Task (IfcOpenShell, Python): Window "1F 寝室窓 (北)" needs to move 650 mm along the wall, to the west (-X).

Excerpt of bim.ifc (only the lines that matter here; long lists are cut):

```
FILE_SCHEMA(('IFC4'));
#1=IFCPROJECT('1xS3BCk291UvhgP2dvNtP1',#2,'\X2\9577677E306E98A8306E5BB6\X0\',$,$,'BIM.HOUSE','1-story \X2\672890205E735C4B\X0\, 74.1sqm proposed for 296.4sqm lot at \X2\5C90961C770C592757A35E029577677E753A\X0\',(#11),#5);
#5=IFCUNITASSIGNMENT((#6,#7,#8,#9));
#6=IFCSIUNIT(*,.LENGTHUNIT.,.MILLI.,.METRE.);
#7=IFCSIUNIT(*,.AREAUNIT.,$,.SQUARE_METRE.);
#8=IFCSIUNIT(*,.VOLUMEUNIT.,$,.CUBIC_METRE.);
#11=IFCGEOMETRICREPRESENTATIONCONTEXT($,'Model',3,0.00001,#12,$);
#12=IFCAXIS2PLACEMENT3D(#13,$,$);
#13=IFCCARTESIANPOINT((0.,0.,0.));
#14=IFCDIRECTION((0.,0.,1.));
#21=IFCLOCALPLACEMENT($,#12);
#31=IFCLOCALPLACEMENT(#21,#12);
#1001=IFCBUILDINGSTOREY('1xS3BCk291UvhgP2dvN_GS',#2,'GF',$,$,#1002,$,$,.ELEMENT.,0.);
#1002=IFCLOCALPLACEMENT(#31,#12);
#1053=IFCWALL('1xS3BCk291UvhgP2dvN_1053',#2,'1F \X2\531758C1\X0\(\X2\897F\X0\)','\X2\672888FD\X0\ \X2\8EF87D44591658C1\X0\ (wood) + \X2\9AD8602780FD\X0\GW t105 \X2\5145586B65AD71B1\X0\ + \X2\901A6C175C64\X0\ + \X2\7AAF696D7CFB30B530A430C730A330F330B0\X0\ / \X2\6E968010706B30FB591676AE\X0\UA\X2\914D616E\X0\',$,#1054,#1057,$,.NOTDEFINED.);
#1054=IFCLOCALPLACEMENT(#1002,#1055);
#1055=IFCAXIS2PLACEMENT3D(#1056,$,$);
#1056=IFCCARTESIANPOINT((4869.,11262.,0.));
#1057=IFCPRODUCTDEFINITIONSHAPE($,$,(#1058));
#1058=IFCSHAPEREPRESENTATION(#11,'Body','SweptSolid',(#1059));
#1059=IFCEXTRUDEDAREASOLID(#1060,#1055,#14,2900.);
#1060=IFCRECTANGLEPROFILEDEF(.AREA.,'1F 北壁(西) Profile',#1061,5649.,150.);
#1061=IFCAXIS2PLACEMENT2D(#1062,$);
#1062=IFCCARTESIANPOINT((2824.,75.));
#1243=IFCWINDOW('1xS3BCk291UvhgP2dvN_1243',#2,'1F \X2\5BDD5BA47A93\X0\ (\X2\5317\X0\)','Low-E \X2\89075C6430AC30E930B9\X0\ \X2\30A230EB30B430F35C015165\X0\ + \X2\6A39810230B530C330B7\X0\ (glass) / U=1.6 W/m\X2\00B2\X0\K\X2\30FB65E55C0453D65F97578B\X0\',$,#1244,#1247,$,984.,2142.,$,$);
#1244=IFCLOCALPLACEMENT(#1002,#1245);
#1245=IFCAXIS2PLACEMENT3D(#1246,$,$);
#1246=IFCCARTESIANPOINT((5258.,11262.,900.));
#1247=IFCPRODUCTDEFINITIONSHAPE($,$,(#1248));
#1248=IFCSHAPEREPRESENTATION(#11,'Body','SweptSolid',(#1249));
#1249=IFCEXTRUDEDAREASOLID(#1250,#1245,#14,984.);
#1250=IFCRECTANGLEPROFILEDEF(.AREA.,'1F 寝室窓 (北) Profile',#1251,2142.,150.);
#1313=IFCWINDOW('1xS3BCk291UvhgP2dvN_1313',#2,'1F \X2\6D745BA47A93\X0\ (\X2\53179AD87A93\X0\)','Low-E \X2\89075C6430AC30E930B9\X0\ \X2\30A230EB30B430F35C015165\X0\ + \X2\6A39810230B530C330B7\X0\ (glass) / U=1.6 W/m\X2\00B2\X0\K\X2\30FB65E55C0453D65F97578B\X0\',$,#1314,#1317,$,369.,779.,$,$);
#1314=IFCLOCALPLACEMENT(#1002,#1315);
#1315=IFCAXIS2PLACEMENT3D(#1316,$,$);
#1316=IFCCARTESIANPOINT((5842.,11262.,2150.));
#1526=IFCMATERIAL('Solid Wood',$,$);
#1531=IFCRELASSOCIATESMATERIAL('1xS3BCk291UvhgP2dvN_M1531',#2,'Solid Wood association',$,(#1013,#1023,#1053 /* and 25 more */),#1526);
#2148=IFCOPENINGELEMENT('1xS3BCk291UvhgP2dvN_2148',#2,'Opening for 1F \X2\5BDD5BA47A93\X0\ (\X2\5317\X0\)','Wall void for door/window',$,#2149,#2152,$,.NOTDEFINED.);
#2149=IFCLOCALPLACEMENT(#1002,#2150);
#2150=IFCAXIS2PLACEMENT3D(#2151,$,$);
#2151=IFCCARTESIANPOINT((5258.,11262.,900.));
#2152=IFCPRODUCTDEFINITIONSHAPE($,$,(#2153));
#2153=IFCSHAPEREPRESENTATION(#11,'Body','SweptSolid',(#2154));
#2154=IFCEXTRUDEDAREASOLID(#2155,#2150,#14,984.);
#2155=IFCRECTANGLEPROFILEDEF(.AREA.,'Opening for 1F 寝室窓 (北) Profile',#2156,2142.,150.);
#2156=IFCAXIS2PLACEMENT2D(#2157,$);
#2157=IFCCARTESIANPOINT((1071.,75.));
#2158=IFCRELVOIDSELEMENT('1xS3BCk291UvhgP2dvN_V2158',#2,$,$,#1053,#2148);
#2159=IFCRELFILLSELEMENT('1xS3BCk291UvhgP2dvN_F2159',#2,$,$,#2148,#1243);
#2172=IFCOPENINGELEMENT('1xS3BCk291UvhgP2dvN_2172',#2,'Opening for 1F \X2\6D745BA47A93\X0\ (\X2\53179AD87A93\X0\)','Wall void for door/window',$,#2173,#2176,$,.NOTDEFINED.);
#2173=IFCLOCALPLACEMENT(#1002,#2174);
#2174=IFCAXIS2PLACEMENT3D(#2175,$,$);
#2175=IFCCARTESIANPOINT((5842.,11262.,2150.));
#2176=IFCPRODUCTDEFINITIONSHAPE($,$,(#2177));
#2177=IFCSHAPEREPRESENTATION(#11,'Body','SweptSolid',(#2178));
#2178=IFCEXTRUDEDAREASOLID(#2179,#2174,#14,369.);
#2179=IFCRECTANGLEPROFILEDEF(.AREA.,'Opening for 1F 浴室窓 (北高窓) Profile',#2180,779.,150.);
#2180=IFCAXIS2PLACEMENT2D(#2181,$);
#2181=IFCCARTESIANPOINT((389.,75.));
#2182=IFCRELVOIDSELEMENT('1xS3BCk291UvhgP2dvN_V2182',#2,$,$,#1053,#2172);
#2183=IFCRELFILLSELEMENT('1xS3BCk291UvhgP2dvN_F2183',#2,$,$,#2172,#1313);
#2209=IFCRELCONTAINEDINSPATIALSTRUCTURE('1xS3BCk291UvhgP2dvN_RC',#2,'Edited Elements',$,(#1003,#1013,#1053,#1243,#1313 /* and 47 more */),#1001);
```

```python
import ifcopenshell
import ifcopenshell.api.geometry
import ifcopenshell.util.placement
import ifcopenshell.util.unit

model = ifcopenshell.open("bim.ifc")
unit_scale = ifcopenshell.util.unit.calculate_unit_scale(model)

window = model.by_guid("1xS3BCk291UvhgP2dvN_1243")
opening = window.FillsVoids[0].RelatingOpeningElement
wall = opening.VoidsElements[0].RelatingBuildingElement

wall_matrix = ifcopenshell.util.placement.get_local_placement(wall.ObjectPlacement)
shift = wall_matrix[:3, 0] * -0.65 / unit_scale
before = ifcopenshell.util.placement.get_local_placement(window.ObjectPlacement)[:3, 3].copy()

# The window is not placed relative to its opening, so move both.
for product in (opening, window):
    matrix = ifcopenshell.util.placement.get_local_placement(product.ObjectPlacement)
    matrix[:3, 3] += shift
    ifcopenshell.api.geometry.edit_object_placement(model, product=product, matrix=matrix, is_si=False)

after = ifcopenshell.util.placement.get_local_placement(window.ObjectPlacement)[:3, 3]
print("window moved by", (after - before).round(3) + 0.0)

model.write("bim_updated.ifc")
```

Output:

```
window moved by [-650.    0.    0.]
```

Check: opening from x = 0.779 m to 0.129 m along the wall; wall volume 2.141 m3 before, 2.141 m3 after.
